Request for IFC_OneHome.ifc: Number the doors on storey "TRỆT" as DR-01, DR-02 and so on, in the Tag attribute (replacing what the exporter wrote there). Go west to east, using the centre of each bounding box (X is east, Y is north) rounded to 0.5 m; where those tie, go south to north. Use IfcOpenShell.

First a look at what the model holds.

```python
import ifcopenshell
import ifcopenshell.util.element
import ifcopenshell.util.placement

model = ifcopenshell.open("IFC_OneHome.ifc")
print(model.schema)
storey = next(s for s in model.by_type("IfcBuildingStorey") if s.Name == "TRỆT")
doors = [e for e in ifcopenshell.util.element.get_decomposition(storey) if e.is_a("IfcDoor")]
for e in sorted(doors, key=lambda e: e.id()):
    origin = ifcopenshell.util.placement.get_local_placement(e.ObjectPlacement)[:3, 3]
    print(e.id(), e.Tag, e.Name, origin.round(2) + 0.0, sep=" | ")
```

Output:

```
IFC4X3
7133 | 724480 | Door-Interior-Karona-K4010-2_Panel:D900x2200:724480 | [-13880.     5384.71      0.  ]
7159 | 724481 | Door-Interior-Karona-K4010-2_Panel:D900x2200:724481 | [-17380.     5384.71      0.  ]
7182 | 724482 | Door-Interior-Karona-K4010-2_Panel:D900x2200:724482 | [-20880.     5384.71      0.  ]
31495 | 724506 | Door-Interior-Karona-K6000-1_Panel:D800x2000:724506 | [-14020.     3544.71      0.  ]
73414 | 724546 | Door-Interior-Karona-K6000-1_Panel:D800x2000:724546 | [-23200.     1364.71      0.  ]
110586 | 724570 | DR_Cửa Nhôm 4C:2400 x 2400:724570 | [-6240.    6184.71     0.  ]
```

```python
import ifcopenshell
import ifcopenshell.geom
import ifcopenshell.util.element
import ifcopenshell.util.shape

model = ifcopenshell.open("IFC_OneHome.ifc")
settings = ifcopenshell.geom.settings()
settings.set("use-world-coords", True)


def centre(element):
    shape = ifcopenshell.geom.create_shape(settings, element)
    return ifcopenshell.util.shape.get_bbox_centroid(shape.geometry)


storey = next(s for s in model.by_type("IfcBuildingStorey") if s.Name == "TRỆT")
doors = [e for e in ifcopenshell.util.element.get_decomposition(storey) if e.is_a("IfcDoor")]

# Insertion points can sit at a corner or the storey origin, so sort by the geometry (in metres).
centres = {e: centre(e) for e in doors}
doors.sort(key=lambda e: (round(centres[e][0] / 0.5), centres[e][1]))

for i, e in enumerate(doors, start=1):
    number = f"DR-{i:02d}"
    e.Tag = number
    print(e.id(), number)

model.write("IFC_OneHome_rev.ifc")
```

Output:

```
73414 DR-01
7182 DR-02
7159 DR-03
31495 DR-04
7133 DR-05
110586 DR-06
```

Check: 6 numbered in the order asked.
